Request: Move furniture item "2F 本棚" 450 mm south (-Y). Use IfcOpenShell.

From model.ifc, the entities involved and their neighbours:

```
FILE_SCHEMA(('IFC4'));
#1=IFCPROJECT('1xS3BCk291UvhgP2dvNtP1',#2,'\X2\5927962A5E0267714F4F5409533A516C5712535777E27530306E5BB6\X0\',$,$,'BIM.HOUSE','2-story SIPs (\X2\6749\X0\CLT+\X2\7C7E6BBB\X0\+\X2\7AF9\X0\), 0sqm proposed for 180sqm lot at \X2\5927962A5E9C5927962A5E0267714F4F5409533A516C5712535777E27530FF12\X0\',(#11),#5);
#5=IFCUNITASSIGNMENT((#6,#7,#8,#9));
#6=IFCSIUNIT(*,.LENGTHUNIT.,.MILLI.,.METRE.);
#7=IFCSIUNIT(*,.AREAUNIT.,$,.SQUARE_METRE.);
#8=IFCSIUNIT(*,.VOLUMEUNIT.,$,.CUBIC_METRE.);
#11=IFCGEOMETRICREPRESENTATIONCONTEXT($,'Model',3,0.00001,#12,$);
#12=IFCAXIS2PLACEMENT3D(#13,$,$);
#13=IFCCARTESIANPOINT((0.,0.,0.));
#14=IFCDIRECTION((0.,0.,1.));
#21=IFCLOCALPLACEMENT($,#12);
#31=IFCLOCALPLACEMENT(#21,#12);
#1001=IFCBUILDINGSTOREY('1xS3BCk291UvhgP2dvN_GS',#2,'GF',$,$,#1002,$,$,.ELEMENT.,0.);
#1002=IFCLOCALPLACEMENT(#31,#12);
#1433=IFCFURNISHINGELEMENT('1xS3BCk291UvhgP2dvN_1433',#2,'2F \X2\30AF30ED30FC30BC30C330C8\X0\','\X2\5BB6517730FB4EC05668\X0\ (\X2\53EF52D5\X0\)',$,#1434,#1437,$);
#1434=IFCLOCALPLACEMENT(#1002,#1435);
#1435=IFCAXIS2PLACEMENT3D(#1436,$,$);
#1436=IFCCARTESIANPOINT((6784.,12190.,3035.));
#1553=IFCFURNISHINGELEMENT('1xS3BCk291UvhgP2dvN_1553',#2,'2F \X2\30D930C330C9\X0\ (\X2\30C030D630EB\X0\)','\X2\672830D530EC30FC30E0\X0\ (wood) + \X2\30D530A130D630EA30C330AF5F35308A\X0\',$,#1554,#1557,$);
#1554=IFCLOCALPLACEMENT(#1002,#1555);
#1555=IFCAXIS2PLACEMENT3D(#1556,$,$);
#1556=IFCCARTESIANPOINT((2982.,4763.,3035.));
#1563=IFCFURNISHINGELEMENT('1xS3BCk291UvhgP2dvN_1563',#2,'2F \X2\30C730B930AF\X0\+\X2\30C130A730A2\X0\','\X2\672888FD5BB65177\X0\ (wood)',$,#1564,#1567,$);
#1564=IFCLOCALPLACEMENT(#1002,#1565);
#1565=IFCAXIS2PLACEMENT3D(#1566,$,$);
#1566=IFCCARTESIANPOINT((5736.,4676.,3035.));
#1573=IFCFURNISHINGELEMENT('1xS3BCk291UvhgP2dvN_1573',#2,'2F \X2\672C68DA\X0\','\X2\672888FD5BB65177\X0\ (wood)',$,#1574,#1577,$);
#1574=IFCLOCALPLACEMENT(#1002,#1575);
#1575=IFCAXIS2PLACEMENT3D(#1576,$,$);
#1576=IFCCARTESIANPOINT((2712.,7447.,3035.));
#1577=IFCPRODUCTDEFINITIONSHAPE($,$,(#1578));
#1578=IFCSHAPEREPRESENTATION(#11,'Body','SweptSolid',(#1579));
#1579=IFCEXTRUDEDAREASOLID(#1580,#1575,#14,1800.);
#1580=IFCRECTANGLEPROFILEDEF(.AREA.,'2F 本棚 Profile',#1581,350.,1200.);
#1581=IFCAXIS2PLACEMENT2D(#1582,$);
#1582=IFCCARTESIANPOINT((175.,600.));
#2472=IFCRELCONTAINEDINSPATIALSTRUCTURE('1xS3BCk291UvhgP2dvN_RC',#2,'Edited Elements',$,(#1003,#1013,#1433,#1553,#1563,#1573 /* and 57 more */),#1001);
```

```python
import ifcopenshell
import ifcopenshell.api.geometry
import ifcopenshell.util.placement
import ifcopenshell.util.unit

model = ifcopenshell.open("model.ifc")
unit_scale = ifcopenshell.util.unit.calculate_unit_scale(model)

item = model.by_guid("1xS3BCk291UvhgP2dvN_1573")
matrix = ifcopenshell.util.placement.get_local_placement(item.ObjectPlacement)
matrix[1, 3] -= 0.45 / unit_scale
ifcopenshell.api.geometry.edit_object_placement(model, product=item, matrix=matrix, is_si=False)

print(ifcopenshell.util.placement.get_local_placement(item.ObjectPlacement).round(3) + 0.0)

model.write("model_edited.ifc")
```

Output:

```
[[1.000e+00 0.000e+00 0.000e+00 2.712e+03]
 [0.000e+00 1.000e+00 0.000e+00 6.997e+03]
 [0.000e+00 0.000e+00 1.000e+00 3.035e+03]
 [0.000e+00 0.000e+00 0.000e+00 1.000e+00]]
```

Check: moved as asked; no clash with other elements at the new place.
